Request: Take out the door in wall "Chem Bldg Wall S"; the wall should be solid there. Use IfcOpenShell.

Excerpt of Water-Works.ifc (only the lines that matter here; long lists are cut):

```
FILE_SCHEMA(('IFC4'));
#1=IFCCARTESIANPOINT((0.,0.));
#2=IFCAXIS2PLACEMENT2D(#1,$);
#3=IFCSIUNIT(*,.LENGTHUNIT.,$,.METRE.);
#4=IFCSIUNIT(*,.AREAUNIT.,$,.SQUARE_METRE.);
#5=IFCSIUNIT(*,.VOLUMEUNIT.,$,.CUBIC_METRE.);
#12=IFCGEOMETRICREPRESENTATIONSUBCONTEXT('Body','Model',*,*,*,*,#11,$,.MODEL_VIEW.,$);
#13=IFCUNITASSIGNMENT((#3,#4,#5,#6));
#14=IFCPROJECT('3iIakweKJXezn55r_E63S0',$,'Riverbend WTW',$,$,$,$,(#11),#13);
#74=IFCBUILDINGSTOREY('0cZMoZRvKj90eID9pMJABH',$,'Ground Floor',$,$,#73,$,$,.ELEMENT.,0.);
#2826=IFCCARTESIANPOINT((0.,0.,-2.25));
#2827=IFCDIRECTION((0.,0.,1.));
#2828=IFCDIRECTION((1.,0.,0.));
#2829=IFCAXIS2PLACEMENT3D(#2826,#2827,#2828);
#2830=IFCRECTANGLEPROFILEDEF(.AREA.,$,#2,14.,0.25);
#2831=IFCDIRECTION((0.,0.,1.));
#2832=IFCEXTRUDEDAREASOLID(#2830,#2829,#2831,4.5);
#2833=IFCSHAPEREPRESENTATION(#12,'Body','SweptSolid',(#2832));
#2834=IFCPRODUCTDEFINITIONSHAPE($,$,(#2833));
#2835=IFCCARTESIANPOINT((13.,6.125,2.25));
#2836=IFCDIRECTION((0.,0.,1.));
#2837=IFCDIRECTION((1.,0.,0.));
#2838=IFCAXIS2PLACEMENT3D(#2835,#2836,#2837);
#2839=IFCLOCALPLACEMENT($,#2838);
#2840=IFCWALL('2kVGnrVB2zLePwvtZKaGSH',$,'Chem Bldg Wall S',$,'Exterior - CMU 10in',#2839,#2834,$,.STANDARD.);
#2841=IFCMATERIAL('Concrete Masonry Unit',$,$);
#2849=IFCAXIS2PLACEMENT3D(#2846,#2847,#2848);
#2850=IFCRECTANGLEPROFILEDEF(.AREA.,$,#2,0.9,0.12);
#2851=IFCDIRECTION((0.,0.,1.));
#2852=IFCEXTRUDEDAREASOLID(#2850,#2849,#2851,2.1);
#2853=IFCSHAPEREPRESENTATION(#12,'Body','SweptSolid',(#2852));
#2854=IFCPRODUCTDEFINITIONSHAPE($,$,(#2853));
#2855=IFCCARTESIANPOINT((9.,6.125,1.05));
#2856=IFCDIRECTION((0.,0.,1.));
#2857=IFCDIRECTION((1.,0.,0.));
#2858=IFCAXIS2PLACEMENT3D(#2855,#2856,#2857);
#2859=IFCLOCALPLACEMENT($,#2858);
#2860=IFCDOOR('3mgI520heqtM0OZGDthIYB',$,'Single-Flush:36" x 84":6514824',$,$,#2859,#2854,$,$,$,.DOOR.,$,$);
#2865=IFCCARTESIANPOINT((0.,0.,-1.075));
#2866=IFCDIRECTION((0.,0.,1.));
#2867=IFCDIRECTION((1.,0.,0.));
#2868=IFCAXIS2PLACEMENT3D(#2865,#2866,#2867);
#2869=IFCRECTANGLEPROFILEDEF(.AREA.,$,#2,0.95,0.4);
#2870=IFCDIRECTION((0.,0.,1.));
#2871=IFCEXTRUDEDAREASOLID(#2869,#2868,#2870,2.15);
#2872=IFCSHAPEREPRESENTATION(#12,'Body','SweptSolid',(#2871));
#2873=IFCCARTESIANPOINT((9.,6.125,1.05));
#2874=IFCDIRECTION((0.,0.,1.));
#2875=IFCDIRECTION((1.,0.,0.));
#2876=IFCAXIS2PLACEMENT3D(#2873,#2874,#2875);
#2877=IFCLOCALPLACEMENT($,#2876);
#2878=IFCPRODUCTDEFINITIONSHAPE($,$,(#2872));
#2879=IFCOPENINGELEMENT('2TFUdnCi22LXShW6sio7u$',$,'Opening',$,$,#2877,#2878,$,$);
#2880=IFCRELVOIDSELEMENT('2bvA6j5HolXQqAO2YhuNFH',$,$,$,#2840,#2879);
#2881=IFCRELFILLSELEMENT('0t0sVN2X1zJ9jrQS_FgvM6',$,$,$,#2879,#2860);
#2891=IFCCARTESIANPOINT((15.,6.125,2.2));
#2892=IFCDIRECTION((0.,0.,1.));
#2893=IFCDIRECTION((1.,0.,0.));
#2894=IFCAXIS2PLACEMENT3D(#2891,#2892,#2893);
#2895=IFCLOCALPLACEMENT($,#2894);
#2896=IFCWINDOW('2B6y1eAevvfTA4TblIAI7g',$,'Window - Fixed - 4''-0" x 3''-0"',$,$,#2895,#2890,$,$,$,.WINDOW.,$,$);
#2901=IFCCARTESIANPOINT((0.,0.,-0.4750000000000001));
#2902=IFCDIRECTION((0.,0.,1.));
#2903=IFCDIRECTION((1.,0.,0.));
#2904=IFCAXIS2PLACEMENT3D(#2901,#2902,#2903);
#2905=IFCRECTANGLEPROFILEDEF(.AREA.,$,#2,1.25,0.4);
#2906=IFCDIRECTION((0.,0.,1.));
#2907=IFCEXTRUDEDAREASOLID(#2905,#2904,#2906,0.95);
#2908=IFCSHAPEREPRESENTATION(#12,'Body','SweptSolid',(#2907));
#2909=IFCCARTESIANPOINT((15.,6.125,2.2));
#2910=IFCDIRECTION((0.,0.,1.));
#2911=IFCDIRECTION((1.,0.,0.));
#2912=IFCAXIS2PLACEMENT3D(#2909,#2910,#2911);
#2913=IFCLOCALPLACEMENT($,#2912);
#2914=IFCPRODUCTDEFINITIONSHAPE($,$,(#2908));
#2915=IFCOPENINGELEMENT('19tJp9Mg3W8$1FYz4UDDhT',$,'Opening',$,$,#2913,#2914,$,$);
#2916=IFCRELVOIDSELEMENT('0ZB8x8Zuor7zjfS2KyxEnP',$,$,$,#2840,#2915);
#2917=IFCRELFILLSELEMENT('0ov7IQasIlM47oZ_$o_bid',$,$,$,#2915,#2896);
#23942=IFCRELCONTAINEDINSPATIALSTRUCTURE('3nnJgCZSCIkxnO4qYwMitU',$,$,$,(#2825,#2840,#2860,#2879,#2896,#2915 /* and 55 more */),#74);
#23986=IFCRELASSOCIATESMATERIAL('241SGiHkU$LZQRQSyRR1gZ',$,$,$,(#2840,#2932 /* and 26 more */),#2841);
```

```python
import ifcopenshell
import ifcopenshell.api.feature
import ifcopenshell.api.root
import ifcopenshell.geom
import ifcopenshell.util.shape

model = ifcopenshell.open("Water-Works.ifc")
settings = ifcopenshell.geom.settings()


def volume(element):
    """Net volume in cubic metres, openings subtracted."""
    shape = ifcopenshell.geom.create_shape(settings, element)
    return ifcopenshell.util.shape.get_volume(shape.geometry)


door = model.by_guid("3mgI520heqtM0OZGDthIYB")
opening = door.FillsVoids[0].RelatingOpeningElement
wall = opening.VoidsElements[0].RelatingBuildingElement
before = volume(wall)

ifcopenshell.api.root.remove_product(model, product=door)
ifcopenshell.api.feature.remove_feature(model, feature=opening)

after = volume(wall)

print(f"wall volume {before:.3f} -> {after:.3f} m3")

model.write("Water-Works_rev.ifc")
```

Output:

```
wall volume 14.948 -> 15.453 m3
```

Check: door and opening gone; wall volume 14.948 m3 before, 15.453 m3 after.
